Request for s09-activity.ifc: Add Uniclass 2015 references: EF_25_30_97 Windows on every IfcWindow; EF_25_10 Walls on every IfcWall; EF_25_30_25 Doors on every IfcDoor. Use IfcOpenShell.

First a look at what the model holds.

```python
import ifcopenshell

model = ifcopenshell.open("s09-activity.ifc")
print(model.schema)
print("classifications:", [c.Name for c in model.by_type("IfcClassification")])
for ifc_class in ("IfcDoor", "IfcRoof", "IfcStair", "IfcWall", "IfcWindow"):
    print(ifc_class, len(model.by_type(ifc_class)))
```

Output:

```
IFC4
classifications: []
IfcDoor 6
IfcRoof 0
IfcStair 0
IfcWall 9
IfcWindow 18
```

```python
import ifcopenshell
import ifcopenshell.api.classification

model = ifcopenshell.open("s09-activity.ifc")

system = ifcopenshell.api.classification.add_classification(model, classification="Uniclass 2015")

codes = {
    "IfcWindow": ("EF_25_30_97", "Windows"),
    "IfcWall": ("EF_25_10", "Walls"),
    "IfcDoor": ("EF_25_30_25", "Doors"),
}
for ifc_class, (code, name) in codes.items():
    products = model.by_type(ifc_class)
    ifcopenshell.api.classification.add_reference(
        model, products=products, classification=system, identification=code, name=name
    )
    print(code, len(products))

model.write("s09-activity_v2.ifc")
```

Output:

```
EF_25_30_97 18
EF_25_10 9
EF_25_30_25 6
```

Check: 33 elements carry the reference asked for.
